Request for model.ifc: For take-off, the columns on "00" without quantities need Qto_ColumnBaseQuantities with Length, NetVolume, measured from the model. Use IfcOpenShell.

First a look at what the model holds.

```python
import ifcopenshell
import ifcopenshell.util.element
import ifcopenshell.util.unit

model = ifcopenshell.open("model.ifc")
print(model.schema)
for unit_type in ("LENGTHUNIT", "AREAUNIT", "VOLUMEUNIT"):
    print(unit_type, ifcopenshell.util.unit.calculate_unit_scale(model, unit_type))
storey = next(s for s in model.by_type("IfcBuildingStorey") if s.Name == "00")
columns = [e for e in ifcopenshell.util.element.get_decomposition(storey) if e.is_a("IfcColumn")]
for e in sorted(columns, key=lambda e: e.id()):
    print(e.id(), e.is_a(), e.Name, list(ifcopenshell.util.element.get_psets(e, qtos_only=True)), sep=" | ")
```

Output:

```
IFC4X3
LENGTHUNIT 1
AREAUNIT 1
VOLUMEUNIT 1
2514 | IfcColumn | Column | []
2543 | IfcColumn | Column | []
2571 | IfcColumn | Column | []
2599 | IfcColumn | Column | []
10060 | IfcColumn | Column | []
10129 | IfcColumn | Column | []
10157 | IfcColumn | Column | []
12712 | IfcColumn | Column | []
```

```python
import ifcopenshell
import ifcopenshell.api.pset
import ifcopenshell.geom
import ifcopenshell.util.element
import ifcopenshell.util.shape
import ifcopenshell.util.unit

model = ifcopenshell.open("model.ifc")
unit_scale = ifcopenshell.util.unit.calculate_unit_scale(model)
volume_scale = ifcopenshell.util.unit.calculate_unit_scale(model, "VOLUMEUNIT")
settings = ifcopenshell.geom.settings()

storey = next(s for s in model.by_type("IfcBuildingStorey") if s.Name == "00")
columns = [e for e in ifcopenshell.util.element.get_decomposition(storey) if e.is_a("IfcColumn")]

for e in sorted(columns, key=lambda e: e.id()):
    if ifcopenshell.util.element.get_psets(e, qtos_only=True, should_inherit=False):
        continue
    # Geometry comes back in metres, in the element's own axes.
    shape = ifcopenshell.geom.create_shape(settings, e)
    values = {
        "Length": ifcopenshell.util.shape.get_z(shape.geometry) / unit_scale,
        "NetVolume": ifcopenshell.util.shape.get_volume(shape.geometry) / volume_scale,
    }
    qto = ifcopenshell.api.pset.add_qto(model, product=e, name="Qto_ColumnBaseQuantities")
    ifcopenshell.api.pset.edit_qto(model, qto=qto, properties=values)
    print(e.id(), {k: round(v, 3) for k, v in values.items()})

model.write("model_v2.ifc")
```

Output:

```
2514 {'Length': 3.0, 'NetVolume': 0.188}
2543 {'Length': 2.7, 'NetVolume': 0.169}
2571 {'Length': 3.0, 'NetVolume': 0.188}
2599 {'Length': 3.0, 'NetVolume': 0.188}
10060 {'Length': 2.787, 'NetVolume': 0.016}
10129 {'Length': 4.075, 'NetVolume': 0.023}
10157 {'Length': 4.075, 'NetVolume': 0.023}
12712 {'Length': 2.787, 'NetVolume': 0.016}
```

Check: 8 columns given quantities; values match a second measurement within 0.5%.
